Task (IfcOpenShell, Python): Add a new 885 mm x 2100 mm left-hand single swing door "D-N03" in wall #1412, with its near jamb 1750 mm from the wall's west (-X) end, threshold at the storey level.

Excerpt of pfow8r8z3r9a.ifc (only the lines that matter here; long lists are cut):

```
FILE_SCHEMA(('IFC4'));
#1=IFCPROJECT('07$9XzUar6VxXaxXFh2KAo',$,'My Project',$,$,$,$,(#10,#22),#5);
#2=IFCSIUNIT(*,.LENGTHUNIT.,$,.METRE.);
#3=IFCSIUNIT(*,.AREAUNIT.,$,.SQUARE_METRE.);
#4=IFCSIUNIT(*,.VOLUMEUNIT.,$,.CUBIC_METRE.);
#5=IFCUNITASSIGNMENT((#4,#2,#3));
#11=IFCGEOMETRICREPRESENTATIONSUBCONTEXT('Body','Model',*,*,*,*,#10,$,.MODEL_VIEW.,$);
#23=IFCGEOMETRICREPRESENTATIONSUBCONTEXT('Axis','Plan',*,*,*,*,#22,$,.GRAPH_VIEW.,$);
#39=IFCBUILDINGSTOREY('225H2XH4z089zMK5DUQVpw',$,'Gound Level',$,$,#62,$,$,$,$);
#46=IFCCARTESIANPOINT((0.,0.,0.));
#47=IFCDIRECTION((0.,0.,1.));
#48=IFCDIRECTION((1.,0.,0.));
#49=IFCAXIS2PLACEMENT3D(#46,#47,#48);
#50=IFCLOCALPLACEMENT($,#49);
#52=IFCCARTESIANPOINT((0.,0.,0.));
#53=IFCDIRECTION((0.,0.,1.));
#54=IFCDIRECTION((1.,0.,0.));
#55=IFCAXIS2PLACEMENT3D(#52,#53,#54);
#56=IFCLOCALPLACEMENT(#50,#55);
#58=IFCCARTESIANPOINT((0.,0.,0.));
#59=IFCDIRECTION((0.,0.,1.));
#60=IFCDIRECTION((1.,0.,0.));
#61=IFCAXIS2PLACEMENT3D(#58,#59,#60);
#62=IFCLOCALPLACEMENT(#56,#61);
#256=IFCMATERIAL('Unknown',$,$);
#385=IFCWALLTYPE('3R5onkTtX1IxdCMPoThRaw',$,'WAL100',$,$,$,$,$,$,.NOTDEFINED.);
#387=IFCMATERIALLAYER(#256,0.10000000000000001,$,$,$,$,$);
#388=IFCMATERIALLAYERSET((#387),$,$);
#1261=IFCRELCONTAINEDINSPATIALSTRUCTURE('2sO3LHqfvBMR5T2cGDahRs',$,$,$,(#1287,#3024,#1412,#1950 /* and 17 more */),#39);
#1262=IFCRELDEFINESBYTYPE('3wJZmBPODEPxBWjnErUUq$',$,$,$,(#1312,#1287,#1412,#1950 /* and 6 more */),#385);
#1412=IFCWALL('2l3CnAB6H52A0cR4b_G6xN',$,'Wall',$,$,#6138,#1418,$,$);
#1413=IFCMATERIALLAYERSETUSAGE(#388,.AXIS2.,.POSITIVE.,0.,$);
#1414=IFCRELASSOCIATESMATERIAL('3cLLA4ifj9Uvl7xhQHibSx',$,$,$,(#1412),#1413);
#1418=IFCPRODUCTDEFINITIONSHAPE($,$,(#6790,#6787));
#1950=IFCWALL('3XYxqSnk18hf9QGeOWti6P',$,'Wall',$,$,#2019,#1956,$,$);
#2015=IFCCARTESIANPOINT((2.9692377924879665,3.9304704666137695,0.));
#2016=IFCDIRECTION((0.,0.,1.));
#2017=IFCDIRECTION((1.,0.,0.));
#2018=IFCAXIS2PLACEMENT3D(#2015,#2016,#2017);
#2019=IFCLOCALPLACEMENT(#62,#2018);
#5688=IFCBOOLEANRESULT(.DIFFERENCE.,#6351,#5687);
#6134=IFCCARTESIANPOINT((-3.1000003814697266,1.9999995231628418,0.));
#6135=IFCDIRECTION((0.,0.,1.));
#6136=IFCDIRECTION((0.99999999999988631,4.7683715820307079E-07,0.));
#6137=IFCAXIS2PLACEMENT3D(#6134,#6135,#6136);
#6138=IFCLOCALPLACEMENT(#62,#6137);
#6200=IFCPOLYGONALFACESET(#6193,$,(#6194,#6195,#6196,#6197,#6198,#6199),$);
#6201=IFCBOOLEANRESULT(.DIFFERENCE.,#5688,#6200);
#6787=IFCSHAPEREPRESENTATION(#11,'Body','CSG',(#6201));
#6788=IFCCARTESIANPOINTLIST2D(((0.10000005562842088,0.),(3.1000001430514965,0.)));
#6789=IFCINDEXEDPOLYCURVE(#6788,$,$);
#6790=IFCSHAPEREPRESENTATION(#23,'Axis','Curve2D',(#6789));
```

```python
import numpy as np
import ifcopenshell
import ifcopenshell.api.feature
import ifcopenshell.api.geometry
import ifcopenshell.api.root
import ifcopenshell.api.spatial
import ifcopenshell.geom
import ifcopenshell.util.element
import ifcopenshell.util.placement
import ifcopenshell.util.representation
import ifcopenshell.util.shape
import ifcopenshell.util.unit

model = ifcopenshell.open("pfow8r8z3r9a.ifc")
unit_scale = ifcopenshell.util.unit.calculate_unit_scale(model)
settings = ifcopenshell.geom.settings()


def volume(element):
    """Net volume in cubic metres, openings subtracted."""
    shape = ifcopenshell.geom.create_shape(settings, element)
    return ifcopenshell.util.shape.get_volume(shape.geometry)


wall = model.by_guid("2l3CnAB6H52A0cR4b_G6xN")
storey = ifcopenshell.util.element.get_container(wall, ifc_class="IfcBuildingStorey")
context = ifcopenshell.util.representation.get_context(model, "Model", "Body", "MODEL_VIEW")
before = volume(wall)

width, height, from_end, sill = 0.885, 2.1, 1.75, 0.0  # metres

# The wall runs along its own X axis, and the end named is its -X end.
wall_shape = ifcopenshell.geom.create_shape(settings, wall)
x, y, z = ifcopenshell.util.shape.get_vertices(wall_shape.geometry).T
start = x.min() + from_end
face, thickness = float(y.min()), float(y.max() - y.min())
wall_matrix = ifcopenshell.util.placement.get_local_placement(wall.ObjectPlacement)
level = ifcopenshell.util.placement.get_local_placement(storey.ObjectPlacement)[2, 3]


def in_wall(x, y):
    """Placement at x, y metres in the wall's axes, at sill height."""
    matrix = wall_matrix.copy()
    matrix[:, 3] = wall_matrix @ np.array([x / unit_scale, y / unit_scale, 0.0, 1.0])
    matrix[2, 3] = level + sill / unit_scale
    return matrix


# Opening: a box that overshoots both wall faces by 50 mm.
opening = ifcopenshell.api.root.create_entity(model, ifc_class="IfcOpeningElement", predefined_type="OPENING")
box = ifcopenshell.api.geometry.add_wall_representation(
    model, context=context, length=width, height=height, thickness=thickness + 0.1
)
ifcopenshell.api.geometry.assign_representation(model, product=opening, representation=box)
ifcopenshell.api.geometry.edit_object_placement(model, product=opening, matrix=in_wall(start, face - 0.05), is_si=False)
ifcopenshell.api.feature.add_feature(model, feature=opening, element=wall)

door = ifcopenshell.api.root.create_entity(model, ifc_class="IfcDoor", name="D-N03", predefined_type="DOOR")
door.OverallWidth, door.OverallHeight = width / unit_scale, height / unit_scale
door.OperationType = "SINGLE_SWING_LEFT"
body = ifcopenshell.api.geometry.add_door_representation(
    model,
    context=context,
    overall_width=door.OverallWidth,
    overall_height=door.OverallHeight,
    operation_type="SINGLE_SWING_LEFT",
    lining_properties={"LiningDepth": thickness / unit_scale, "ThresholdDepth": thickness / unit_scale},
)
ifcopenshell.api.geometry.assign_representation(model, product=door, representation=body)
ifcopenshell.api.spatial.assign_container(model, products=[door], relating_structure=storey)
ifcopenshell.api.feature.add_filling(model, opening=opening, element=door)

# The lining spans the wall, so the door starts at the wall face.
ifcopenshell.api.geometry.edit_object_placement(model, product=door, matrix=in_wall(start, face), is_si=False)

after = volume(wall)

print(f"wall volume {before:.3f} -> {after:.3f} m3")

model.write("pfow8r8z3r9a_rev.ifc")
```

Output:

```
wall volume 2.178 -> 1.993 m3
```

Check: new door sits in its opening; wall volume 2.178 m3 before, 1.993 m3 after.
